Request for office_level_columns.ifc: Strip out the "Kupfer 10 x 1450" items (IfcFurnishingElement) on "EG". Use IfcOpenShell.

First a look at what the model holds.

```python
import ifcopenshell
import ifcopenshell.util.element

model = ifcopenshell.open("office_level_columns.ifc")
print(model.schema)
storey = next(s for s in model.by_type("IfcBuildingStorey") if s.Name == "EG")
furniture = [e for e in ifcopenshell.util.element.get_decomposition(storey) if e.is_a("IfcFurnishingElement")]
seen = {}
for e in furniture:
    element_type = ifcopenshell.util.element.get_type(e)
    name = element_type.Name if element_type not in (None, e) else None
    seen[name] = seen.get(name, 0) + 1
for name, count in sorted(seen.items(), key=str):
    print(count, "x", name)
```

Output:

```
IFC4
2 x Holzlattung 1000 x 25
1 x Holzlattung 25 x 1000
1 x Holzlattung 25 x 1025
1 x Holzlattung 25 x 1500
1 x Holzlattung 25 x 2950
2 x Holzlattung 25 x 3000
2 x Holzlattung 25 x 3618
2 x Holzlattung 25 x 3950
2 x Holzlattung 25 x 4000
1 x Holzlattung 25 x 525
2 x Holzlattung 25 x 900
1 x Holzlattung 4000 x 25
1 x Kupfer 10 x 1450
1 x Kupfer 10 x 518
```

```python
import ifcopenshell
import ifcopenshell.api.root
import ifcopenshell.util.element

model = ifcopenshell.open("office_level_columns.ifc")

storey = next(s for s in model.by_type("IfcBuildingStorey") if s.Name == "EG")
furniture = [e for e in ifcopenshell.util.element.get_decomposition(storey) if e.is_a("IfcFurnishingElement")]
targets = [e for e in furniture if (t := ifcopenshell.util.element.get_type(e)) not in (None, e) and t.Name == "Kupfer 10 x 1450"]

for e in targets:
    ifcopenshell.api.root.remove_product(model, product=e)
print(len(targets), "removed")

model.write("office_level_columns_v2.ifc")
```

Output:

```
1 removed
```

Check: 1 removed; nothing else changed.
